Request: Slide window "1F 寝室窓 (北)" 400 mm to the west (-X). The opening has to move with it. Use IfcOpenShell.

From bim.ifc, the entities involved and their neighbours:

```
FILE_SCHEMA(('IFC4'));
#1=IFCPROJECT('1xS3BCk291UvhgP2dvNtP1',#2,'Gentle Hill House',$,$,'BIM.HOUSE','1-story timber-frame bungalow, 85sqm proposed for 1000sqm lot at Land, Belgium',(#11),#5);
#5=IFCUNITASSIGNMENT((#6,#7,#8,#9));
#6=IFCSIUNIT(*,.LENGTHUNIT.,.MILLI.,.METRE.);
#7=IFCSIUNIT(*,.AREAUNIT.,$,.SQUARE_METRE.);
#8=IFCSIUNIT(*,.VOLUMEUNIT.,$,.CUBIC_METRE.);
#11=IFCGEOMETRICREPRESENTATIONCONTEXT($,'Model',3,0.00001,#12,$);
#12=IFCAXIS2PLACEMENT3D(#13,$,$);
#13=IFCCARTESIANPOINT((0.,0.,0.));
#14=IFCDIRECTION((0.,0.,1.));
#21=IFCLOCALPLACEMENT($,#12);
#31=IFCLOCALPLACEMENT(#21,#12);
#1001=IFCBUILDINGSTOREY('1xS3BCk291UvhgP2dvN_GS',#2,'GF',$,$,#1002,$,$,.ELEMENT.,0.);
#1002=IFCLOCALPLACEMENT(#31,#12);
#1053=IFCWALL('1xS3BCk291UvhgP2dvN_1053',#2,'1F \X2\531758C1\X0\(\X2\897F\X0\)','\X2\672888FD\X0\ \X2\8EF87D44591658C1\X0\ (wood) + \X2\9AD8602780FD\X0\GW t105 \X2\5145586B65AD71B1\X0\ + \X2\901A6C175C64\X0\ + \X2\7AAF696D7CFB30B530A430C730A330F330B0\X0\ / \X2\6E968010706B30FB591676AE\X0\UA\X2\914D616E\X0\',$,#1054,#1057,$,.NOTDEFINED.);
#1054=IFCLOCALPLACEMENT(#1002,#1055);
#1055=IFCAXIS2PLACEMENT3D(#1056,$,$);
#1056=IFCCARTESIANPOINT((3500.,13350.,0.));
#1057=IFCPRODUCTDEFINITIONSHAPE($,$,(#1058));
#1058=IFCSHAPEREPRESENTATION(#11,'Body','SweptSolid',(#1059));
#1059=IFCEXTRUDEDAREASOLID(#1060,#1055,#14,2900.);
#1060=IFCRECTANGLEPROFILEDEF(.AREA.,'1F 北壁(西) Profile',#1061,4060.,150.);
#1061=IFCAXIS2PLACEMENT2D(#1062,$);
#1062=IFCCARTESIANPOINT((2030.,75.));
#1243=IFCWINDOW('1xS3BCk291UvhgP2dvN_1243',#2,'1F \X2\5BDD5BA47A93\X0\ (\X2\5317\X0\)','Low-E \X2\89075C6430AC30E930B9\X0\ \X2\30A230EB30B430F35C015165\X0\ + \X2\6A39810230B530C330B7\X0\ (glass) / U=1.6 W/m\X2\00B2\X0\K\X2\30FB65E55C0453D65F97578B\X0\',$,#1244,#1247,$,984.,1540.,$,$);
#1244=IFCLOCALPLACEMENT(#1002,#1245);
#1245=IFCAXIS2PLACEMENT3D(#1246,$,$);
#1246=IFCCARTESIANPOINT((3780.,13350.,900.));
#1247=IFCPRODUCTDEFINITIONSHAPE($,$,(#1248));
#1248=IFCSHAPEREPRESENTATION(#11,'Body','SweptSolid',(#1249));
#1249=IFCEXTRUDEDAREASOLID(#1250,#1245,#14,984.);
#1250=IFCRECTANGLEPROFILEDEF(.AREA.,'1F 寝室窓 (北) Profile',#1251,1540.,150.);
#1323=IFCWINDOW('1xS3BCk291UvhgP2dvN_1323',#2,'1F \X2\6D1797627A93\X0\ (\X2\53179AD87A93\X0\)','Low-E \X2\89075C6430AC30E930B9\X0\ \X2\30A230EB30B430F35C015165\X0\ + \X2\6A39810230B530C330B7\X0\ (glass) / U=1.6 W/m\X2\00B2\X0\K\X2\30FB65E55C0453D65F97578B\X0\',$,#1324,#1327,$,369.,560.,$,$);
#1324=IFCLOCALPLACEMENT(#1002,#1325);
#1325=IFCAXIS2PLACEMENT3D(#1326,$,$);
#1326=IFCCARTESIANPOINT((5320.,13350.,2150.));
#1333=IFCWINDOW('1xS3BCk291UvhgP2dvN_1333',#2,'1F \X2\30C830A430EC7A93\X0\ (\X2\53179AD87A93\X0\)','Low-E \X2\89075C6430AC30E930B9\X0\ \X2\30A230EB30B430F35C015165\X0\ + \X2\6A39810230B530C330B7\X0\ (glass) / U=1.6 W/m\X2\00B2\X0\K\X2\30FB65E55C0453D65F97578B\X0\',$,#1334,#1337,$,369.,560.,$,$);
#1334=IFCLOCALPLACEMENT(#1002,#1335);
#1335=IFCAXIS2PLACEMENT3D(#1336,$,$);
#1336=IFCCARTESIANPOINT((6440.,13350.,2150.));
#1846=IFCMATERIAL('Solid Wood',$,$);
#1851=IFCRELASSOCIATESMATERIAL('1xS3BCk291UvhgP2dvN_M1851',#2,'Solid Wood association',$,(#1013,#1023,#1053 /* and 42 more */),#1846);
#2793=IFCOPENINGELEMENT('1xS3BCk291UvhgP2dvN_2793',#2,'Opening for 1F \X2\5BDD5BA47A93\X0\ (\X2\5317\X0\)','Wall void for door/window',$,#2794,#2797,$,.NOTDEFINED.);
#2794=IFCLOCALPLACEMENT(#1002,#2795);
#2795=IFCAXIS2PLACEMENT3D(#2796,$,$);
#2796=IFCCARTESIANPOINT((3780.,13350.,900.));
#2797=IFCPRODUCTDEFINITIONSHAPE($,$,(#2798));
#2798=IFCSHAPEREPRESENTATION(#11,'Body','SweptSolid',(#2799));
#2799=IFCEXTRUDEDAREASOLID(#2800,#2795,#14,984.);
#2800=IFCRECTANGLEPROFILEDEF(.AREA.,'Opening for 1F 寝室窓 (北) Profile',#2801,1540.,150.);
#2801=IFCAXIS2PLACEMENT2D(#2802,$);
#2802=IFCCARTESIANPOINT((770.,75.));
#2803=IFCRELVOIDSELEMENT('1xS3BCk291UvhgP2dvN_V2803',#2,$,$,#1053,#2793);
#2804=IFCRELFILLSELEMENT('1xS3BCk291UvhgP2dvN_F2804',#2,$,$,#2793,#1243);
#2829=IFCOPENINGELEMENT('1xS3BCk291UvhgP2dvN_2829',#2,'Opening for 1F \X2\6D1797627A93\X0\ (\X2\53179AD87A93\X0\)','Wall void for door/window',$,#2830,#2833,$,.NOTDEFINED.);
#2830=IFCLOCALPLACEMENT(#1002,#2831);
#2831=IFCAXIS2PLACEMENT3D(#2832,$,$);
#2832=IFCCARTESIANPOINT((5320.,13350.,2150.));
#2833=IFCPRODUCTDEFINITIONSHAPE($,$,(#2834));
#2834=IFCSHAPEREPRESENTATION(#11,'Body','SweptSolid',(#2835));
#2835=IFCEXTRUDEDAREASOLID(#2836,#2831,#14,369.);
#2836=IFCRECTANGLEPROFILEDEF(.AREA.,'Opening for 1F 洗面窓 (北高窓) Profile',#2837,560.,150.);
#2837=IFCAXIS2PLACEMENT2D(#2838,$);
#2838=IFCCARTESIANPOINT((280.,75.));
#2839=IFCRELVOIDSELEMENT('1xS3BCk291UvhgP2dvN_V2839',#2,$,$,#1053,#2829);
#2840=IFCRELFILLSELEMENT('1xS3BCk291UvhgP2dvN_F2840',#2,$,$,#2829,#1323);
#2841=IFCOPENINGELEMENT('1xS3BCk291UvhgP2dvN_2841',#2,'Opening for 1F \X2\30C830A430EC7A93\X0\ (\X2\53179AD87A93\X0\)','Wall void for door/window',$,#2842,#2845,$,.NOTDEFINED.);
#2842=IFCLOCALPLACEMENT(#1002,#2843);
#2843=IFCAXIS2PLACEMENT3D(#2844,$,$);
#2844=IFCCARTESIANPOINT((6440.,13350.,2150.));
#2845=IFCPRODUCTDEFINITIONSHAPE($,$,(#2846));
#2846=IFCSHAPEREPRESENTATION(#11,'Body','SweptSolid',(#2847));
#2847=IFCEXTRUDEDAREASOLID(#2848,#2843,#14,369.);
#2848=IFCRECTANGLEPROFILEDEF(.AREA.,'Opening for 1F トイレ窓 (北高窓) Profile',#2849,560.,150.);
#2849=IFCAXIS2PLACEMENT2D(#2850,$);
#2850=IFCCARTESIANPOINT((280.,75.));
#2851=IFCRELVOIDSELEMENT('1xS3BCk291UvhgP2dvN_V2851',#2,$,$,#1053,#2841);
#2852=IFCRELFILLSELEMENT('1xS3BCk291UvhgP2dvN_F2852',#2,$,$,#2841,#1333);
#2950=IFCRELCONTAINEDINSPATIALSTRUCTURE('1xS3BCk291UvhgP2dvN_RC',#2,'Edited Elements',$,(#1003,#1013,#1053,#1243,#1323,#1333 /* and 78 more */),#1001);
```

```python
import ifcopenshell
import ifcopenshell.api.geometry
import ifcopenshell.util.placement
import ifcopenshell.util.unit

model = ifcopenshell.open("bim.ifc")
unit_scale = ifcopenshell.util.unit.calculate_unit_scale(model)

window = model.by_guid("1xS3BCk291UvhgP2dvN_1243")
opening = window.FillsVoids[0].RelatingOpeningElement
wall = opening.VoidsElements[0].RelatingBuildingElement

wall_matrix = ifcopenshell.util.placement.get_local_placement(wall.ObjectPlacement)
shift = wall_matrix[:3, 0] * -0.4 / unit_scale
before = ifcopenshell.util.placement.get_local_placement(window.ObjectPlacement)[:3, 3].copy()

# The window is not placed relative to its opening, so move both.
for product in (opening, window):
    matrix = ifcopenshell.util.placement.get_local_placement(product.ObjectPlacement)
    matrix[:3, 3] += shift
    ifcopenshell.api.geometry.edit_object_placement(model, product=product, matrix=matrix, is_si=False)

after = ifcopenshell.util.placement.get_local_placement(window.ObjectPlacement)[:3, 3]
print("window moved by", (after - before).round(3) + 0.0)

model.write("bim_updated.ifc")
```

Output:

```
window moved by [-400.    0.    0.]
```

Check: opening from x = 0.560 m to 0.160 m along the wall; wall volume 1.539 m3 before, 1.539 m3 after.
